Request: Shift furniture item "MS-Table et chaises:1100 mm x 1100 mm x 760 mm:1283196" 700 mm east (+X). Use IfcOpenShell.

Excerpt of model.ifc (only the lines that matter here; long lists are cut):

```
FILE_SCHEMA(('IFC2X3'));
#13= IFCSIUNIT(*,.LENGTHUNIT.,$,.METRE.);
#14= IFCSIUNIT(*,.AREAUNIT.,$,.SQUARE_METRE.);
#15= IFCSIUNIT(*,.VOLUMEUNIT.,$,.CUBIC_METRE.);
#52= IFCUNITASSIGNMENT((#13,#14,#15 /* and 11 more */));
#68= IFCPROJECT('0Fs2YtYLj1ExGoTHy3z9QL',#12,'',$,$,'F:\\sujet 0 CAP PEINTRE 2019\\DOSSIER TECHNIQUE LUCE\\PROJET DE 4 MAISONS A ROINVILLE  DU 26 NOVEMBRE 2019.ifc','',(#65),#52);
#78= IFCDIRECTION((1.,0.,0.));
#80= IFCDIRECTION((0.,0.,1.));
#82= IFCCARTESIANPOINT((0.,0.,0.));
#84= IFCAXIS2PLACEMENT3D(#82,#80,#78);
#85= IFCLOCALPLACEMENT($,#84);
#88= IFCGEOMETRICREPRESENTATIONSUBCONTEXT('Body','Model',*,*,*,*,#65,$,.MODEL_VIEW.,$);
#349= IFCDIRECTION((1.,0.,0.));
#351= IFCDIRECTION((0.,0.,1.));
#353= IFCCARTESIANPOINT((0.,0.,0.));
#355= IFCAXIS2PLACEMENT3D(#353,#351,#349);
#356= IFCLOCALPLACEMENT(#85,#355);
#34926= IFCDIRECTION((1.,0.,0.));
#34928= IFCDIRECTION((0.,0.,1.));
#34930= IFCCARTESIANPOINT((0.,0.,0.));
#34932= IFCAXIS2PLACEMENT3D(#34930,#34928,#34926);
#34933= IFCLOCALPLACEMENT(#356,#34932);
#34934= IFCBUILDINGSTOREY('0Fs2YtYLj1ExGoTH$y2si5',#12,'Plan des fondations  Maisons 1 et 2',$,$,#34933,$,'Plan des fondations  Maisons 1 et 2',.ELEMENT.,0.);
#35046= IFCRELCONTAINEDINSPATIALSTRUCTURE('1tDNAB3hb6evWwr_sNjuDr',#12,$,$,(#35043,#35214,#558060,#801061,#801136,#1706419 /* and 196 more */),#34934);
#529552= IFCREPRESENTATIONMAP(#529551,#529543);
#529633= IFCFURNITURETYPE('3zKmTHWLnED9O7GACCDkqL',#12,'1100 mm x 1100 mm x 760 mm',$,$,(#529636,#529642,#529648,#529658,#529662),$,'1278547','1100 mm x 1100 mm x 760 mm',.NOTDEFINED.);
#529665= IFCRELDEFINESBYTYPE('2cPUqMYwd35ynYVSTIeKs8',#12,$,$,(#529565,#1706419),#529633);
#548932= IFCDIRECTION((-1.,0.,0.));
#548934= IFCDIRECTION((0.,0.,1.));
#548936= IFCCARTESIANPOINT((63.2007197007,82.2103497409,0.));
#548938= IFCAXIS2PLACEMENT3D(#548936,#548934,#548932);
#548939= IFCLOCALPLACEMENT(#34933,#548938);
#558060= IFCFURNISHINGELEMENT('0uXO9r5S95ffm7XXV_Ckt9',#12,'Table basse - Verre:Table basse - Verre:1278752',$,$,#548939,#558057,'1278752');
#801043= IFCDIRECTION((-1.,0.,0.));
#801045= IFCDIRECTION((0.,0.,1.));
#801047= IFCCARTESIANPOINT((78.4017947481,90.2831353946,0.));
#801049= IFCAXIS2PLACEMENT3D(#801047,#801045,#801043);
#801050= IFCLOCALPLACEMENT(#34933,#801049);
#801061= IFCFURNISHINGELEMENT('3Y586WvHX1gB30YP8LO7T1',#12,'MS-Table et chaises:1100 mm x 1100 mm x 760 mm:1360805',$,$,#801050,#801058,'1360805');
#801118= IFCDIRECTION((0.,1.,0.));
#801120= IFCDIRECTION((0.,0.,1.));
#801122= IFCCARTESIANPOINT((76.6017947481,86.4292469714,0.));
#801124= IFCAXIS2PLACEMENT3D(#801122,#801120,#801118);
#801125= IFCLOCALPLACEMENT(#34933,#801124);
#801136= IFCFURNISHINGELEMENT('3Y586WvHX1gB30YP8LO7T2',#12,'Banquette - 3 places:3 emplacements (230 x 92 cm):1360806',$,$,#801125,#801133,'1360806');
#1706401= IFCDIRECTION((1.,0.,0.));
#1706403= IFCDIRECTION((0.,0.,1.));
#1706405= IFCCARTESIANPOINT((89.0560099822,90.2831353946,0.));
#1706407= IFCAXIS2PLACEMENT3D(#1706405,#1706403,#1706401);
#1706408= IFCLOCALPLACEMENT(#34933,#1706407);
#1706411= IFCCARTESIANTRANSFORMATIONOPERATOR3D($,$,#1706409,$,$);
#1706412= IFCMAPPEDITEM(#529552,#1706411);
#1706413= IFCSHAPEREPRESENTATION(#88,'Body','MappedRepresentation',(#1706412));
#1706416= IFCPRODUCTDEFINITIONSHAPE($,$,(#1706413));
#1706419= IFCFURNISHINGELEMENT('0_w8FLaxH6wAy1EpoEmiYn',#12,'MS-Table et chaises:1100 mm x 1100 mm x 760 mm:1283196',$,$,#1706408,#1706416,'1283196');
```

```python
import ifcopenshell
import ifcopenshell.api.geometry
import ifcopenshell.util.placement
import ifcopenshell.util.unit

model = ifcopenshell.open("model.ifc")
unit_scale = ifcopenshell.util.unit.calculate_unit_scale(model)

item = model.by_guid("0_w8FLaxH6wAy1EpoEmiYn")
matrix = ifcopenshell.util.placement.get_local_placement(item.ObjectPlacement)
matrix[0, 3] += 0.7 / unit_scale
ifcopenshell.api.geometry.edit_object_placement(model, product=item, matrix=matrix, is_si=False)

print(ifcopenshell.util.placement.get_local_placement(item.ObjectPlacement).round(3) + 0.0)

model.write("model-out.ifc")
```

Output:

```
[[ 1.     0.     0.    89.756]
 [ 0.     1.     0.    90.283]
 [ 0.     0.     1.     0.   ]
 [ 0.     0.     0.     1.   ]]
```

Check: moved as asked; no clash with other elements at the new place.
